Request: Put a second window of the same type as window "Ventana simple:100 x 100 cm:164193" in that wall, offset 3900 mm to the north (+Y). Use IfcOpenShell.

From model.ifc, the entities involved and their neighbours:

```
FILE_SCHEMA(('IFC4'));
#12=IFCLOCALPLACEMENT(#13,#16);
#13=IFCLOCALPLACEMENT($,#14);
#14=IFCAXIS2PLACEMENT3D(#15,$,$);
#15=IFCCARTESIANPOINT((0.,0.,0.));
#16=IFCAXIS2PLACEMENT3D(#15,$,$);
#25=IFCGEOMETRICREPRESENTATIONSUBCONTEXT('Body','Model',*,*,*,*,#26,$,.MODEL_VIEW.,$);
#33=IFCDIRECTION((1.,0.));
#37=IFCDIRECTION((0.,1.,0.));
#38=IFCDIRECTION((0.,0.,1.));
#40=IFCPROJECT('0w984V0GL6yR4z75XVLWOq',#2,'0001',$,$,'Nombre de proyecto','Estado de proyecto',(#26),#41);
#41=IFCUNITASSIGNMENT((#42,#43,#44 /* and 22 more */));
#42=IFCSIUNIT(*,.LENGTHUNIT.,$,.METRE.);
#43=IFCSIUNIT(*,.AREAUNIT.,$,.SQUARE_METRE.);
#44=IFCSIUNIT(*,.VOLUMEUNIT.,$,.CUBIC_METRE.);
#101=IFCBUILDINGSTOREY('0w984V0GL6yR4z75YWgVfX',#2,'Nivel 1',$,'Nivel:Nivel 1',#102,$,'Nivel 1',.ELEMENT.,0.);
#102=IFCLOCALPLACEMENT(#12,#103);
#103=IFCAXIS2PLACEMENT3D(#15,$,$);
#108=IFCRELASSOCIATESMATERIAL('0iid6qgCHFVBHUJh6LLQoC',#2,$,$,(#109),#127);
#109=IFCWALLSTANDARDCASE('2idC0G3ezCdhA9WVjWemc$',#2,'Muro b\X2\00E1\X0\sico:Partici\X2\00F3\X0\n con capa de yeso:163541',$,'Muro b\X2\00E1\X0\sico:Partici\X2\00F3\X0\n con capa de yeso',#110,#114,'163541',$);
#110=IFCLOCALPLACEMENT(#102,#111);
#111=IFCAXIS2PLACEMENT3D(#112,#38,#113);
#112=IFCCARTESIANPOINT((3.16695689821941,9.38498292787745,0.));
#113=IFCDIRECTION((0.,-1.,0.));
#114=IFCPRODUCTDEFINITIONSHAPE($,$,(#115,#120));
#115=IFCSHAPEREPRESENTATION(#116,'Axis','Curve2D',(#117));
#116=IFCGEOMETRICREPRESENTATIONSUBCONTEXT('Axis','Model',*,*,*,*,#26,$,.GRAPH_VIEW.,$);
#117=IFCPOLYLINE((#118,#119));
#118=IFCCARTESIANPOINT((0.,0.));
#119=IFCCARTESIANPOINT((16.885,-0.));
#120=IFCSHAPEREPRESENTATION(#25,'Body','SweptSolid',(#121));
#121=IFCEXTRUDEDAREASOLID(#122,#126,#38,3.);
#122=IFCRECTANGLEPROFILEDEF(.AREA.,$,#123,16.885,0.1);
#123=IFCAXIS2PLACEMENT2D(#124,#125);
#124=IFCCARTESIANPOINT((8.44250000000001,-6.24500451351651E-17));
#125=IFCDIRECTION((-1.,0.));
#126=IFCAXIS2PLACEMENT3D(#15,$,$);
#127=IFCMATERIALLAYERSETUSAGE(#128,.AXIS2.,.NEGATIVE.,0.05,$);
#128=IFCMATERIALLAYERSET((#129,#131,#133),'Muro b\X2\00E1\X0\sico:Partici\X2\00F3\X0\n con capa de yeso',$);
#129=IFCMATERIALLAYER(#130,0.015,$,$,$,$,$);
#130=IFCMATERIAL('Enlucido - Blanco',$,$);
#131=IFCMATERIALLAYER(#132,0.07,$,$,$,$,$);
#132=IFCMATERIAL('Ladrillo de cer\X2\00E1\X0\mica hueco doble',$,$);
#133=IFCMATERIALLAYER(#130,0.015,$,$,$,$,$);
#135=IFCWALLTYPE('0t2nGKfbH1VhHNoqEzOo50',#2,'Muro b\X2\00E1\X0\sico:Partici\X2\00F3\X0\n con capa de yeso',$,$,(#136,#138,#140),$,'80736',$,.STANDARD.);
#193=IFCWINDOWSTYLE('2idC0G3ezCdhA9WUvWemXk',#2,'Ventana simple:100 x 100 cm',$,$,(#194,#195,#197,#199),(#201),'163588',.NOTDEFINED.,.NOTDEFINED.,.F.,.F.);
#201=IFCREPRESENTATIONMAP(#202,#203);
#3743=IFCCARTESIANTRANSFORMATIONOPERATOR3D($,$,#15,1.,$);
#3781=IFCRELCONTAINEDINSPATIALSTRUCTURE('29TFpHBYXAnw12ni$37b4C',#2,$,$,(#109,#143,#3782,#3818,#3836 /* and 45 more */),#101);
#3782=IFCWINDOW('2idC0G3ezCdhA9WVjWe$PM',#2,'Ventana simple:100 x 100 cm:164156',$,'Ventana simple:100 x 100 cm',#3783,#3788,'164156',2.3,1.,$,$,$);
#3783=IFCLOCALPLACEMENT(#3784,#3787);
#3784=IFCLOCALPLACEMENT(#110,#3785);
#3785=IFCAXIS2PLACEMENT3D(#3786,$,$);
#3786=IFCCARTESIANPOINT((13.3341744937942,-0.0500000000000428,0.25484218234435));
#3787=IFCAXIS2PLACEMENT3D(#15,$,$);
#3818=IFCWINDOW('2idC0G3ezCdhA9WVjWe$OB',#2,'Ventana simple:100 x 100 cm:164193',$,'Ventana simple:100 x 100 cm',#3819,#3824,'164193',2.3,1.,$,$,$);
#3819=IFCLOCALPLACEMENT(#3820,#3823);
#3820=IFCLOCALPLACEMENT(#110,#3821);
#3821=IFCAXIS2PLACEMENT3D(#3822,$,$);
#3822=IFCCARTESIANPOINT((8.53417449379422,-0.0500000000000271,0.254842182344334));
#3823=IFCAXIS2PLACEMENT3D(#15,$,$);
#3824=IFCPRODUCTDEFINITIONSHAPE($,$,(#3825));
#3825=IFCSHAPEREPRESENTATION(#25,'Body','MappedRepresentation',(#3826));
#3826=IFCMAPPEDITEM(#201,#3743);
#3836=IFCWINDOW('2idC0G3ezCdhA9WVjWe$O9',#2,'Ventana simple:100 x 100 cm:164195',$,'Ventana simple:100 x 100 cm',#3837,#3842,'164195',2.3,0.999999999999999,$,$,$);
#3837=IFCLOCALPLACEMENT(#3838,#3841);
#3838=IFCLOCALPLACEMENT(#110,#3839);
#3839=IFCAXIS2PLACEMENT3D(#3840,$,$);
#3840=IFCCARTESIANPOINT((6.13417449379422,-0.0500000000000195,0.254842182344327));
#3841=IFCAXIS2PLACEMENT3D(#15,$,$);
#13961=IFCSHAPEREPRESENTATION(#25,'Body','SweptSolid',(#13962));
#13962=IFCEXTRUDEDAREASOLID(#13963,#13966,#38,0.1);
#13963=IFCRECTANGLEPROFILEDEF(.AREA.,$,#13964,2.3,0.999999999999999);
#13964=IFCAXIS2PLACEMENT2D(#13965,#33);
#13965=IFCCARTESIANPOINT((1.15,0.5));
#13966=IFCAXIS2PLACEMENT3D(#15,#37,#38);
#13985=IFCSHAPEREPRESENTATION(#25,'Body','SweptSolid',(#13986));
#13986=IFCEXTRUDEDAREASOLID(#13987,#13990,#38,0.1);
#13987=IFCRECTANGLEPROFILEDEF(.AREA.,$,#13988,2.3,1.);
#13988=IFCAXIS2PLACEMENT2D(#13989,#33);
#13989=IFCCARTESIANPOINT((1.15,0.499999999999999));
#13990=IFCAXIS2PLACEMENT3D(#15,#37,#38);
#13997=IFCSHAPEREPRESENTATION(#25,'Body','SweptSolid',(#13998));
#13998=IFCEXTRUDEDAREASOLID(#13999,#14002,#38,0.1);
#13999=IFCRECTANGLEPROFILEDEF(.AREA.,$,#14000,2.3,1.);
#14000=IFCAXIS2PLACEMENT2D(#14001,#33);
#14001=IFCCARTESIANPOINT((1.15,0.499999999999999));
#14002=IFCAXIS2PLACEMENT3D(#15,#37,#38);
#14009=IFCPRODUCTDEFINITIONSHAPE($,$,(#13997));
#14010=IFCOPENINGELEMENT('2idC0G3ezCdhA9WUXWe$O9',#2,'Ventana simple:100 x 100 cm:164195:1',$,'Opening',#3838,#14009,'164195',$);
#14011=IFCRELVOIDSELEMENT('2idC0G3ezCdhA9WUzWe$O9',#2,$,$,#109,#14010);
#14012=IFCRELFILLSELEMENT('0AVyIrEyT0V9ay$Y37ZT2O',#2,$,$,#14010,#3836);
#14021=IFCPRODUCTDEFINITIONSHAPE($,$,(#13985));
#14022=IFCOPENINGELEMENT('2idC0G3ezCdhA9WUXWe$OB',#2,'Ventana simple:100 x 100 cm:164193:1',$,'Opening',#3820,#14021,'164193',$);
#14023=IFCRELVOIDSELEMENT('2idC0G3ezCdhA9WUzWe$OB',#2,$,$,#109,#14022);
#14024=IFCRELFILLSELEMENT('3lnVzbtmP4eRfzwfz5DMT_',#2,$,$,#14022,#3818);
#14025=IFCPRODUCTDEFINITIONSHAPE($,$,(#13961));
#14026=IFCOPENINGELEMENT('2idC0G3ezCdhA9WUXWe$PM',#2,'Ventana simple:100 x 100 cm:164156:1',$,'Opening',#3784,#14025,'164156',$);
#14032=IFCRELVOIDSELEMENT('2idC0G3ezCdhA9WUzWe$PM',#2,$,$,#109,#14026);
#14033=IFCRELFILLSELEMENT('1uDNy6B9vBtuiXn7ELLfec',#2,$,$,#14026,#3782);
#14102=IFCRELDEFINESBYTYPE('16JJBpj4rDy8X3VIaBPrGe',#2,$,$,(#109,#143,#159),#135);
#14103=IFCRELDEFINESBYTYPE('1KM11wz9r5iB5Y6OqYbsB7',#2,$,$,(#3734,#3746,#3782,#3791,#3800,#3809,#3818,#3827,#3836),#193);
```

```python
import ifcopenshell
import ifcopenshell.api.feature
import ifcopenshell.api.geometry
import ifcopenshell.api.root
import ifcopenshell.geom
import ifcopenshell.util.element
import ifcopenshell.util.placement
import ifcopenshell.util.shape

model = ifcopenshell.open("model.ifc")
settings = ifcopenshell.geom.settings()


def volume(element):
    """Net volume in cubic metres, openings subtracted."""
    shape = ifcopenshell.geom.create_shape(settings, element)
    return ifcopenshell.util.shape.get_volume(shape.geometry)


def reuse_history(source, copy):
    """copy_class also copies each property set's owner history, people and application; keep the originals."""
    for rel in copy.IsDefinedBy:
        if rel.is_a("IfcRelDefinesByProperties") and (history := rel.RelatingPropertyDefinition.OwnerHistory):
            rel.RelatingPropertyDefinition.OwnerHistory = source.OwnerHistory
            ifcopenshell.util.element.remove_deep2(model, history)


window = model.by_guid("2idC0G3ezCdhA9WVjWe$OB")
opening = window.FillsVoids[0].RelatingOpeningElement
wall = opening.VoidsElements[0].RelatingBuildingElement
before = volume(wall)
shift = ifcopenshell.util.placement.get_local_placement(wall.ObjectPlacement)[:3, 0] * -3.9

# copy_class copies the void relationship, type, container and properties, but no geometry.
new_opening = ifcopenshell.api.root.copy_class(model, product=opening)
new_opening.Representation = ifcopenshell.util.element.copy_deep(
    model, opening.Representation, exclude=["IfcGeometricRepresentationContext", "IfcRepresentationMap"]
)
new_opening.Name = "Ventana simple:100 x 100 cm"
new_opening.Tag = None
new_window = ifcopenshell.api.root.copy_class(model, product=window)
new_window.Representation = ifcopenshell.util.element.copy_deep(
    model, window.Representation, exclude=["IfcGeometricRepresentationContext", "IfcRepresentationMap"]
)
new_window.Name = "Ventana simple:100 x 100 cm"
new_window.Tag = None
reuse_history(window, new_window)
ifcopenshell.api.feature.add_filling(model, opening=new_opening, element=new_window)

for old, new in ((opening, new_opening), (window, new_window)):
    matrix = ifcopenshell.util.placement.get_local_placement(old.ObjectPlacement)
    matrix[:3, 3] += shift
    ifcopenshell.api.geometry.edit_object_placement(model, product=new, matrix=matrix, is_si=False)

after = volume(wall)

print(f"wall volume {before:.3f} -> {after:.3f} m3")

model.write("model_updated.ifc")
```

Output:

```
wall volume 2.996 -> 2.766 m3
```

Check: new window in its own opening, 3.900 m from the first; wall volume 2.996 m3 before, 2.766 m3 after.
